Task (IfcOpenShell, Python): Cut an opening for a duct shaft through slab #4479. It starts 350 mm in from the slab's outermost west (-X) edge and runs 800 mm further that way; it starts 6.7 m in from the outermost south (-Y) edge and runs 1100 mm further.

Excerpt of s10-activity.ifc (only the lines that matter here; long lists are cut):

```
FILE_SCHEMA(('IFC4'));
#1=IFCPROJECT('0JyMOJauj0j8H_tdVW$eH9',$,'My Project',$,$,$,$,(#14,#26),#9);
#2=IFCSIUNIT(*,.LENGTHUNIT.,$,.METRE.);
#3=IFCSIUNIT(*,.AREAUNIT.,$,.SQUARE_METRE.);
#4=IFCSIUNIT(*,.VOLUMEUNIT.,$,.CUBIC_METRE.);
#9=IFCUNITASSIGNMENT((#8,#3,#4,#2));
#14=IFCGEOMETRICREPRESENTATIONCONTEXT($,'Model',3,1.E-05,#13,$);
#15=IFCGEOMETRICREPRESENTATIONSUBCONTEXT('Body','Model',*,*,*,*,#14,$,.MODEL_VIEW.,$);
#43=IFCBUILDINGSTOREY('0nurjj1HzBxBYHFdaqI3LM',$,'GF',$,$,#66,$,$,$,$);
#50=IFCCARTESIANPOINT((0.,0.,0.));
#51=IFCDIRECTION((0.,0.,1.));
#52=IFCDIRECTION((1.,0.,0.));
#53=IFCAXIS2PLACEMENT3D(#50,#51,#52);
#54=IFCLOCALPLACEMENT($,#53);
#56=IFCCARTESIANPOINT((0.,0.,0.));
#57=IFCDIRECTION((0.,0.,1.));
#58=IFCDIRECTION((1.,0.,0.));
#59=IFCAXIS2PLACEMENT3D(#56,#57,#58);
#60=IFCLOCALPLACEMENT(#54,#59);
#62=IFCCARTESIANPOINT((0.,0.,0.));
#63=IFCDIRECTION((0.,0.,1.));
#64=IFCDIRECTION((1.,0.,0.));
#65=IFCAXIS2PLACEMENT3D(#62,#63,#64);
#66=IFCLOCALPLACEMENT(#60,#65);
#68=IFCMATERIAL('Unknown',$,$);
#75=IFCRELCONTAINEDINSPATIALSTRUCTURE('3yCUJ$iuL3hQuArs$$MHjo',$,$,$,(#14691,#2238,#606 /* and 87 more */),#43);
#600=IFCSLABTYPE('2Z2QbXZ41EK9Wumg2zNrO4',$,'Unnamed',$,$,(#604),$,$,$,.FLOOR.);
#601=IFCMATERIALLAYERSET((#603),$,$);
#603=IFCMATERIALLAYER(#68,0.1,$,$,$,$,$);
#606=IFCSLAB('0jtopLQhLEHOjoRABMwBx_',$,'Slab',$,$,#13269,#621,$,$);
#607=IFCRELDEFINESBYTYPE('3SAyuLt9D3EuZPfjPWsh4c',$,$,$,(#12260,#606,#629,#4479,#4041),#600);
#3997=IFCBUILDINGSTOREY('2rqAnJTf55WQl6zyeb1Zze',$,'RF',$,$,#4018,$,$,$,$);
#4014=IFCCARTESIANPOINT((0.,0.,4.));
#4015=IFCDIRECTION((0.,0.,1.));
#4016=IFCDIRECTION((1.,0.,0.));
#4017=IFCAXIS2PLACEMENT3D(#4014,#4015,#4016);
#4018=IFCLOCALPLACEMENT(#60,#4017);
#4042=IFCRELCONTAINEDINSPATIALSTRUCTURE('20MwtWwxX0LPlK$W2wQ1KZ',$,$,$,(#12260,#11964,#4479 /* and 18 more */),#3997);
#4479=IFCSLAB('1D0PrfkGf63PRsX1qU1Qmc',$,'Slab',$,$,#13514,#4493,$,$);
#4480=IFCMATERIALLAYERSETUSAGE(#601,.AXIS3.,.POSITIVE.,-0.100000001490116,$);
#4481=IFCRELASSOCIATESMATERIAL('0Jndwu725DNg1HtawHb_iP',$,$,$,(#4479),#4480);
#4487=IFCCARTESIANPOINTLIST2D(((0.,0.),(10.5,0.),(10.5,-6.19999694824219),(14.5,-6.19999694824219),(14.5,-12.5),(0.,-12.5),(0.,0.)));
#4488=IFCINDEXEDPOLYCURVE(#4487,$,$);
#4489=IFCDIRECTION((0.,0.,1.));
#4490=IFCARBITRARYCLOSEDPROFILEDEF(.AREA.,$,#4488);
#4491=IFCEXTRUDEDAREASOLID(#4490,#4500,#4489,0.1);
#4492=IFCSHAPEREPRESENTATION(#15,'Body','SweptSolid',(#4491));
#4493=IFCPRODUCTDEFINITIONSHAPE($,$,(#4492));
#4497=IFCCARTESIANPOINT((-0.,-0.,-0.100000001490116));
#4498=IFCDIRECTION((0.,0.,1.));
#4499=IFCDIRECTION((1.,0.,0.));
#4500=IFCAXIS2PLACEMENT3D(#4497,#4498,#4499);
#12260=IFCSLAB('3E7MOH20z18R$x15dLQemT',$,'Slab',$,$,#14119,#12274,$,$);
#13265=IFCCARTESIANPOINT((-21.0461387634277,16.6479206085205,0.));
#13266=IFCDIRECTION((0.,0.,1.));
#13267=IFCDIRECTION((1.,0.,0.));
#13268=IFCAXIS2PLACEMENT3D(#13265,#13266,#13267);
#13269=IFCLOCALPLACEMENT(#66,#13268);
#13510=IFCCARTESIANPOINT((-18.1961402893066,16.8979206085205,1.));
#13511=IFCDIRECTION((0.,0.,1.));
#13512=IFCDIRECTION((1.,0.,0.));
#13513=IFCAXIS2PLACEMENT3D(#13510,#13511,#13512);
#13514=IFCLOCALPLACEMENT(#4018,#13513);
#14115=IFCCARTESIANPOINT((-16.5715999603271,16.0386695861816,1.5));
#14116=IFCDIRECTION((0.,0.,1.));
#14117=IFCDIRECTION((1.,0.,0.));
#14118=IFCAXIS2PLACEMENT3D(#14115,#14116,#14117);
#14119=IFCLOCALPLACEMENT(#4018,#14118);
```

```python
import numpy as np
import ifcopenshell
import ifcopenshell.api.feature
import ifcopenshell.api.geometry
import ifcopenshell.api.root
import ifcopenshell.geom
import ifcopenshell.util.placement
import ifcopenshell.util.representation
import ifcopenshell.util.shape
import ifcopenshell.util.unit

model = ifcopenshell.open("s10-activity.ifc")
unit_scale = ifcopenshell.util.unit.calculate_unit_scale(model)
settings = ifcopenshell.geom.settings()


def volume(element):
    """Net volume in cubic metres, openings subtracted."""
    shape = ifcopenshell.geom.create_shape(settings, element)
    return ifcopenshell.util.shape.get_volume(shape.geometry)


slab = model.by_guid("1D0PrfkGf63PRsX1qU1Qmc")
before = volume(slab)

# Extent in the slab's own axes, in metres. The edges named are its -X and -Y sides.
slab_shape = ifcopenshell.geom.create_shape(settings, slab)
vertices = ifcopenshell.util.shape.get_vertices(slab_shape.geometry)
x_min, y_min, bottom = vertices.min(axis=0)
top = vertices[:, 2].max()

opening = ifcopenshell.api.root.create_entity(model, ifc_class="IfcOpeningElement", name="Duct shaft opening", predefined_type="OPENING")
context = ifcopenshell.util.representation.get_context(model, "Model", "Body", "MODEL_VIEW")
width, depth = 0.8, 1.1
outline = [(0.0, 0.0), (width, 0.0), (width, depth), (0.0, depth), (0.0, 0.0)]
# Overshoot both faces by 50 mm so the cut is clean.
shape = ifcopenshell.api.geometry.add_slab_representation(
    model, context=context, depth=top - bottom + 0.1, polyline=outline
)
ifcopenshell.api.geometry.assign_representation(model, product=opening, representation=shape)

matrix = ifcopenshell.util.placement.get_local_placement(slab.ObjectPlacement)
matrix[:, 3] = matrix @ np.append(np.array([x_min + 0.35, y_min + 6.7, bottom - 0.05]) / unit_scale, 1.0)
ifcopenshell.api.geometry.edit_object_placement(model, product=opening, matrix=matrix, is_si=False)
ifcopenshell.api.feature.add_feature(model, feature=opening, element=slab)

after = volume(slab)

print(f"slab volume {before:.3f} -> {after:.3f} m3")

model.write("s10-activity_updated.ifc")
```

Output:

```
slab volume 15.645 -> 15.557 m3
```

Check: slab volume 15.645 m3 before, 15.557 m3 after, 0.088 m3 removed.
